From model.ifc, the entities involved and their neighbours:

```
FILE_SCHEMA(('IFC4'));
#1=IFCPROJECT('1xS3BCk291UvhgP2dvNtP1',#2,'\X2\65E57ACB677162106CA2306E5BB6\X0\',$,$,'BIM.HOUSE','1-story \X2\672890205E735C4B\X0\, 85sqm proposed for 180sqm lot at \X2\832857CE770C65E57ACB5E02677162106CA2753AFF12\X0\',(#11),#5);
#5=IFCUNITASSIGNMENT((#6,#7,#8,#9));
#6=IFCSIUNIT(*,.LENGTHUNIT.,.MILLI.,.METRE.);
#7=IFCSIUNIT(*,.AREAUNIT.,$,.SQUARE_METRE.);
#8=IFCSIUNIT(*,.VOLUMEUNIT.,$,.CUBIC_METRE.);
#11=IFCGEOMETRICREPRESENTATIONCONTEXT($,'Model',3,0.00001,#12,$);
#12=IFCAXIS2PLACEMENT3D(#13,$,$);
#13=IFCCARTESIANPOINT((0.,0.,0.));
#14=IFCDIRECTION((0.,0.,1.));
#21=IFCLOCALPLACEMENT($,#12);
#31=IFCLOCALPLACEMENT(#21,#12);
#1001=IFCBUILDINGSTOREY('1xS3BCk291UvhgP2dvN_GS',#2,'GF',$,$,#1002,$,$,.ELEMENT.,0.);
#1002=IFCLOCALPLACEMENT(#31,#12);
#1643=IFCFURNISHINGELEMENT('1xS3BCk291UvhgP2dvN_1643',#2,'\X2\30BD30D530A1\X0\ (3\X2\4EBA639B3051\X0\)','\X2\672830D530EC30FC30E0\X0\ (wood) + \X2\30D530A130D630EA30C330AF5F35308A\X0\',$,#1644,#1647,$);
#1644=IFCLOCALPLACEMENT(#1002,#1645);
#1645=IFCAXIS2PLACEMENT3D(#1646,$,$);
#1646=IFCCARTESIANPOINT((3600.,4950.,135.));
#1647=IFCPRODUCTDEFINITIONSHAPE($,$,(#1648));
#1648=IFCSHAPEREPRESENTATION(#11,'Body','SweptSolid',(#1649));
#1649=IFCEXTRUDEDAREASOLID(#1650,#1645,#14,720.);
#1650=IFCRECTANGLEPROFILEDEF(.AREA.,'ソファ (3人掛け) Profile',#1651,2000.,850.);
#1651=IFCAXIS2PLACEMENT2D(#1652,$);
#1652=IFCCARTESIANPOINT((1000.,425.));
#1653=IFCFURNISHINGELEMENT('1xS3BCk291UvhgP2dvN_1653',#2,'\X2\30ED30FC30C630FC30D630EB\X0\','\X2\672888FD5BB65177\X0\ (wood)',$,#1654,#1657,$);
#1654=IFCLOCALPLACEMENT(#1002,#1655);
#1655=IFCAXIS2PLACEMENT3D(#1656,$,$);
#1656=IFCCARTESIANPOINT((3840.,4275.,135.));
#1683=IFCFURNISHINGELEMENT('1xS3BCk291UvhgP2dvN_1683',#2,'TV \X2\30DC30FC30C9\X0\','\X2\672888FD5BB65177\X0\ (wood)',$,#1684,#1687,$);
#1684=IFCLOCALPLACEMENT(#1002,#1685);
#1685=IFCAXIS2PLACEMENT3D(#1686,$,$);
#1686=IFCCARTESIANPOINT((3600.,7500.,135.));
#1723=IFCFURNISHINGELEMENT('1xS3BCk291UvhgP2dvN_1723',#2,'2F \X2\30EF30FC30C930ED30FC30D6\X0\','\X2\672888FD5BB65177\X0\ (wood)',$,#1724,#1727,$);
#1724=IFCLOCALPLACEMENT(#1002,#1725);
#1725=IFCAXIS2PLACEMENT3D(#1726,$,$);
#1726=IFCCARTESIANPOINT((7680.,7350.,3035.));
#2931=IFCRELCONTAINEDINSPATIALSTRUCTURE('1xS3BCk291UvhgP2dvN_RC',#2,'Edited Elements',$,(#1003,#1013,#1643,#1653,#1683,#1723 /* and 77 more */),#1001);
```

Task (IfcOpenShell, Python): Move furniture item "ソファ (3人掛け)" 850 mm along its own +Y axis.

```python
import ifcopenshell
import ifcopenshell.api.geometry
import ifcopenshell.util.placement

model = ifcopenshell.open("model.ifc")

item = model.by_guid("1xS3BCk291UvhgP2dvN_1643")
matrix = ifcopenshell.util.placement.get_local_placement(item.ObjectPlacement)
matrix[:3, 3] += matrix[:3, 1] * 850.0
ifcopenshell.api.geometry.edit_object_placement(model, product=item, matrix=matrix, is_si=False)

print(ifcopenshell.util.placement.get_local_placement(item.ObjectPlacement).round(3) + 0.0)

model.write("model_v2.ifc")
```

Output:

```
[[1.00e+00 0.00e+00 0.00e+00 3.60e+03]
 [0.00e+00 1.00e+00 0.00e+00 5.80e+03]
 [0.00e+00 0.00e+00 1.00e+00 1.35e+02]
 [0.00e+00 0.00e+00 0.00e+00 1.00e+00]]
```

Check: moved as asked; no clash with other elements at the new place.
